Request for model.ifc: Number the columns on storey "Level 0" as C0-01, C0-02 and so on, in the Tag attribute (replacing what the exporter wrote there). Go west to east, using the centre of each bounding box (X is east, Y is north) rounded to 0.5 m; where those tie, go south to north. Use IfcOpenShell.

First a look at what the model holds.

```python
import ifcopenshell
import ifcopenshell.util.element
import ifcopenshell.util.placement

model = ifcopenshell.open("model.ifc")
print(model.schema)
storey = next(s for s in model.by_type("IfcBuildingStorey") if s.Name == "Level 0")
columns = [e for e in ifcopenshell.util.element.get_decomposition(storey) if e.is_a("IfcColumn")]
for e in sorted(columns, key=lambda e: e.id()):
    origin = ifcopenshell.util.placement.get_local_placement(e.ObjectPlacement)[:3, 3]
    print(e.id(), e.Tag, e.Name, origin.round(2) + 0.0, sep=" | ")
```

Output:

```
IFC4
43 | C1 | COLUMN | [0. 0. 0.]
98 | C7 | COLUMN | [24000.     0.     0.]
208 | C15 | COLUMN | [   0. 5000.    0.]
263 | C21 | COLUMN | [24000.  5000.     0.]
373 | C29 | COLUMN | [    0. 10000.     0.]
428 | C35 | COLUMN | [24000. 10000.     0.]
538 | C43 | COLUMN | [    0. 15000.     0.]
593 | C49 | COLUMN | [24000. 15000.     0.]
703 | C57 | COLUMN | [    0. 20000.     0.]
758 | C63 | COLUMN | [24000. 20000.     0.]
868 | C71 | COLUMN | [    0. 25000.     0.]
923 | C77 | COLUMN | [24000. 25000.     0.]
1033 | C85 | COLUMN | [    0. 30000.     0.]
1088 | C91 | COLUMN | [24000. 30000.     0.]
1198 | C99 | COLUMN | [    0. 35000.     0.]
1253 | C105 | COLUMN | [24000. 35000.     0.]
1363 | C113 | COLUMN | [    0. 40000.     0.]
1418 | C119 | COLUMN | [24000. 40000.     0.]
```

```python
import ifcopenshell
import ifcopenshell.geom
import ifcopenshell.util.element
import ifcopenshell.util.shape

model = ifcopenshell.open("model.ifc")
settings = ifcopenshell.geom.settings()
settings.set("use-world-coords", True)


def centre(element):
    shape = ifcopenshell.geom.create_shape(settings, element)
    return ifcopenshell.util.shape.get_bbox_centroid(shape.geometry)


storey = next(s for s in model.by_type("IfcBuildingStorey") if s.Name == "Level 0")
columns = [e for e in ifcopenshell.util.element.get_decomposition(storey) if e.is_a("IfcColumn")]

# Insertion points can sit at a corner or the storey origin, so sort by the geometry (in metres).
centres = {e: centre(e) for e in columns}
columns.sort(key=lambda e: (round(centres[e][0] / 0.5), centres[e][1]))

for i, e in enumerate(columns, start=1):
    number = f"C0-{i:02d}"
    e.Tag = number
    print(e.id(), number)

model.write("model_v2.ifc")
```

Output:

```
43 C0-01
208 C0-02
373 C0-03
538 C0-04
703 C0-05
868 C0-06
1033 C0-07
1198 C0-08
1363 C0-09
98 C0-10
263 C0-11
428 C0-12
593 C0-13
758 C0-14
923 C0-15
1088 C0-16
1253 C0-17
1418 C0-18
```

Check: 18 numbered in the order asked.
